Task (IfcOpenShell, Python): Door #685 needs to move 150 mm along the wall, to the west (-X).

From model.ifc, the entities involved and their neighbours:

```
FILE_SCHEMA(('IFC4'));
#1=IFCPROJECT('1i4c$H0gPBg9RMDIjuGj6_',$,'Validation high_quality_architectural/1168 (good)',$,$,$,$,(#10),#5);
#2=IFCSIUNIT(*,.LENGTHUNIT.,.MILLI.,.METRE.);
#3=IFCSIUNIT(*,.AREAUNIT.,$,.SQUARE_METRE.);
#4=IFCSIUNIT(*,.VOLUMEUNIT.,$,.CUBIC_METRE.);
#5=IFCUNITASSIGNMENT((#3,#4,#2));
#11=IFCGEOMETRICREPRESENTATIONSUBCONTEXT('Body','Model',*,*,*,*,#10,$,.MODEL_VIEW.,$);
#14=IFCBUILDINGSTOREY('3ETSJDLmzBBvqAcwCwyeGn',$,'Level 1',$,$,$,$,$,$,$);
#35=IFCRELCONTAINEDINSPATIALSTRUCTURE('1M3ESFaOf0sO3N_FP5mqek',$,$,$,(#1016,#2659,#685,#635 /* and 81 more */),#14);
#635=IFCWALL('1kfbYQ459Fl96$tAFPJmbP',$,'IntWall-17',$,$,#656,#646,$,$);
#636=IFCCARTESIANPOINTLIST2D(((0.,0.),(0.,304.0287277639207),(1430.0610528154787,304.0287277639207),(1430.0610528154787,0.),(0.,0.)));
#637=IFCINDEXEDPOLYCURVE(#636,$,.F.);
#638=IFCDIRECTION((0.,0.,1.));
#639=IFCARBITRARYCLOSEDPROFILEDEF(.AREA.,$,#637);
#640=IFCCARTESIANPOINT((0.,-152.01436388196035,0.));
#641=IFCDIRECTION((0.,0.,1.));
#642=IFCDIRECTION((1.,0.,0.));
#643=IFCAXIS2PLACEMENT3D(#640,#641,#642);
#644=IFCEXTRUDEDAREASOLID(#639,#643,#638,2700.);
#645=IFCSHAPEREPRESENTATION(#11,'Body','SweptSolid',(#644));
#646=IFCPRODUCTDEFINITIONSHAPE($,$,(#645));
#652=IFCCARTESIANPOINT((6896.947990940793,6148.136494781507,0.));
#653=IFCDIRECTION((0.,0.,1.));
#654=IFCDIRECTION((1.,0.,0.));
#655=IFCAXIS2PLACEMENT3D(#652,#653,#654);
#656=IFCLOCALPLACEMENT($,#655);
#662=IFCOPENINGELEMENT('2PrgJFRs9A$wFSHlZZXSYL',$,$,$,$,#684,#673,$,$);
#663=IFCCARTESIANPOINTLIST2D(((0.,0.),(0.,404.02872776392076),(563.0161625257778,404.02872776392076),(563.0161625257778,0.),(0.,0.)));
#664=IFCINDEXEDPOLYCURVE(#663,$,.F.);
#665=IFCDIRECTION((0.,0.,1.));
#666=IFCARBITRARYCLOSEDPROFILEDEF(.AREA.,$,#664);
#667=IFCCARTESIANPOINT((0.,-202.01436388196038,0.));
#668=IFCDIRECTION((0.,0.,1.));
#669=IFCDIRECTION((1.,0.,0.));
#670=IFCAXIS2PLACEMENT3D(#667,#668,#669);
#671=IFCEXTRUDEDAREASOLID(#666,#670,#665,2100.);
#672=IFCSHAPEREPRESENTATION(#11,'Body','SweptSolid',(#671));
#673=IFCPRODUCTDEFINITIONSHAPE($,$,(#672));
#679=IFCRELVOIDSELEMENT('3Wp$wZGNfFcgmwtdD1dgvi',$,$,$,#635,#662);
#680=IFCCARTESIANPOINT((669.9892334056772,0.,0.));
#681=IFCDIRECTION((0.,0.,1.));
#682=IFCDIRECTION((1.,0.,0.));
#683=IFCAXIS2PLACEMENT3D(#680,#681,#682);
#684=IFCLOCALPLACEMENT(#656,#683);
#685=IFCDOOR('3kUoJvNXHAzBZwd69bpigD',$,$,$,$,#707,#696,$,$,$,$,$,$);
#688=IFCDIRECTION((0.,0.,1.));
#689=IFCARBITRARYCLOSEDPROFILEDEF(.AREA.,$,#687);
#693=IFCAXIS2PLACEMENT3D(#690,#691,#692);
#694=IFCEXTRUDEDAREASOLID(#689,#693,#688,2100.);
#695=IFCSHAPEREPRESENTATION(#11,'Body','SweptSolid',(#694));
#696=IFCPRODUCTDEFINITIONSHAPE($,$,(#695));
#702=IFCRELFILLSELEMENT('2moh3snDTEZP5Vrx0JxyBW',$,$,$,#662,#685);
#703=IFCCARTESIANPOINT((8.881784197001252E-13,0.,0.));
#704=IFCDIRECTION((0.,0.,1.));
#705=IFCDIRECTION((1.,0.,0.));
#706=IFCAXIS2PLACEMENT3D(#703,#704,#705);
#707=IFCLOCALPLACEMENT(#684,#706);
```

```python
import ifcopenshell
import ifcopenshell.api.geometry
import ifcopenshell.util.placement
import ifcopenshell.util.unit

model = ifcopenshell.open("model.ifc")
unit_scale = ifcopenshell.util.unit.calculate_unit_scale(model)

door = model.by_id(685)
opening = door.FillsVoids[0].RelatingOpeningElement
wall = opening.VoidsElements[0].RelatingBuildingElement

wall_matrix = ifcopenshell.util.placement.get_local_placement(wall.ObjectPlacement)
shift = wall_matrix[:3, 0] * -0.15 / unit_scale
before = ifcopenshell.util.placement.get_local_placement(door.ObjectPlacement)[:3, 3].copy()

# The door is placed relative to its opening, so it follows when the opening moves.
matrix = ifcopenshell.util.placement.get_local_placement(opening.ObjectPlacement)
matrix[:3, 3] += shift
ifcopenshell.api.geometry.edit_object_placement(
    model, product=opening, matrix=matrix, is_si=False, should_transform_children=True
)

after = ifcopenshell.util.placement.get_local_placement(door.ObjectPlacement)[:3, 3]
print("door moved by", (after - before).round(3) + 0.0)

model.write("model_updated.ifc")
```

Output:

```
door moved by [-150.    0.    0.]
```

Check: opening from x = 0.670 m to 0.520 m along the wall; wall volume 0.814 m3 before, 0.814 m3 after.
